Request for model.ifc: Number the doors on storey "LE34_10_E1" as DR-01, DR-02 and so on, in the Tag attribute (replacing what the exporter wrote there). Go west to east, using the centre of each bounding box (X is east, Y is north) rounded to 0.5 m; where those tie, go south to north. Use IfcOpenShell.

First a look at what the model holds.

```python
import ifcopenshell
import ifcopenshell.util.element
import ifcopenshell.util.placement

model = ifcopenshell.open("model.ifc")
print(model.schema)
storey = next(s for s in model.by_type("IfcBuildingStorey") if s.Name == "LE34_10_E1")
doors = [e for e in ifcopenshell.util.element.get_decomposition(storey) if e.is_a("IfcDoor")]
for e in sorted(doors, key=lambda e: e.id()):
    origin = ifcopenshell.util.placement.get_local_placement(e.ObjectPlacement)[:3, 3]
    print(e.id(), e.Tag, e.Name, origin.round(2) + 0.0, sep=" | ")
```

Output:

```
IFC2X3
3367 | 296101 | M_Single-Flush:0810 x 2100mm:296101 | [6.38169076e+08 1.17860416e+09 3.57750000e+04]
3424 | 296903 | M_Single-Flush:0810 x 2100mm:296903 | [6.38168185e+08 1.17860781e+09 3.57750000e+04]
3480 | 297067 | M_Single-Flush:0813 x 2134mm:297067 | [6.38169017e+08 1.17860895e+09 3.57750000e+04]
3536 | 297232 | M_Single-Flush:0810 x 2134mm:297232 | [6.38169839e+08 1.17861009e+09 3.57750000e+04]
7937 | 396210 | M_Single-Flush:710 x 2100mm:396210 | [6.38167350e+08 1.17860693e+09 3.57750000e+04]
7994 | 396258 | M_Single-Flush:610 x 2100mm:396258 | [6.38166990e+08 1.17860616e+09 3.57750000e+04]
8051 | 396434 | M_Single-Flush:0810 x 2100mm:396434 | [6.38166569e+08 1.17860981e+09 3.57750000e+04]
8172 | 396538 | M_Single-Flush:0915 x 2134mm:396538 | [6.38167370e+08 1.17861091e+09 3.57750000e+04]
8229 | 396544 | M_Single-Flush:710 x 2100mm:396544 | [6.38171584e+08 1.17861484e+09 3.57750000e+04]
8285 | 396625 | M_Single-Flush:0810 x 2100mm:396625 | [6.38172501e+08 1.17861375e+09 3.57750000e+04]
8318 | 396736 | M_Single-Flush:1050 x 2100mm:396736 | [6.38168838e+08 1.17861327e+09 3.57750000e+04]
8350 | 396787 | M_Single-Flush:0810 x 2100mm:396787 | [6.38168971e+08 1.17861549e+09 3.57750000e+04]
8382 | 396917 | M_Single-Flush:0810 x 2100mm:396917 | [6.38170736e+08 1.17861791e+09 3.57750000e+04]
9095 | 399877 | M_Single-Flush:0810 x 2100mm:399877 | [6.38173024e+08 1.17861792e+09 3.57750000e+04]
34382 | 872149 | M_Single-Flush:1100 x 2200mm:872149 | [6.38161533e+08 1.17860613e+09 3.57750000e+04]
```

```python
import ifcopenshell
import ifcopenshell.geom
import ifcopenshell.util.element
import ifcopenshell.util.shape

model = ifcopenshell.open("model.ifc")
settings = ifcopenshell.geom.settings()
settings.set("use-world-coords", True)


def centre(element):
    shape = ifcopenshell.geom.create_shape(settings, element)
    return ifcopenshell.util.shape.get_bbox_centroid(shape.geometry)


storey = next(s for s in model.by_type("IfcBuildingStorey") if s.Name == "LE34_10_E1")
doors = [e for e in ifcopenshell.util.element.get_decomposition(storey) if e.is_a("IfcDoor")]

# Insertion points can sit at a corner or the storey origin, so sort by the geometry (in metres).
centres = {e: centre(e) for e in doors}
doors.sort(key=lambda e: (round(centres[e][0] / 0.5), centres[e][1]))

for i, e in enumerate(doors, start=1):
    number = f"DR-{i:02d}"
    e.Tag = number
    print(e.id(), number)

model.write("model_rev.ifc")
```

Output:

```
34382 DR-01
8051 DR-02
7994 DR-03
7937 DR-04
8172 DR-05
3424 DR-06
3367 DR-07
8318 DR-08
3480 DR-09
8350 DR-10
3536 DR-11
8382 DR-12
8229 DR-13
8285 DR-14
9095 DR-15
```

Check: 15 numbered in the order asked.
